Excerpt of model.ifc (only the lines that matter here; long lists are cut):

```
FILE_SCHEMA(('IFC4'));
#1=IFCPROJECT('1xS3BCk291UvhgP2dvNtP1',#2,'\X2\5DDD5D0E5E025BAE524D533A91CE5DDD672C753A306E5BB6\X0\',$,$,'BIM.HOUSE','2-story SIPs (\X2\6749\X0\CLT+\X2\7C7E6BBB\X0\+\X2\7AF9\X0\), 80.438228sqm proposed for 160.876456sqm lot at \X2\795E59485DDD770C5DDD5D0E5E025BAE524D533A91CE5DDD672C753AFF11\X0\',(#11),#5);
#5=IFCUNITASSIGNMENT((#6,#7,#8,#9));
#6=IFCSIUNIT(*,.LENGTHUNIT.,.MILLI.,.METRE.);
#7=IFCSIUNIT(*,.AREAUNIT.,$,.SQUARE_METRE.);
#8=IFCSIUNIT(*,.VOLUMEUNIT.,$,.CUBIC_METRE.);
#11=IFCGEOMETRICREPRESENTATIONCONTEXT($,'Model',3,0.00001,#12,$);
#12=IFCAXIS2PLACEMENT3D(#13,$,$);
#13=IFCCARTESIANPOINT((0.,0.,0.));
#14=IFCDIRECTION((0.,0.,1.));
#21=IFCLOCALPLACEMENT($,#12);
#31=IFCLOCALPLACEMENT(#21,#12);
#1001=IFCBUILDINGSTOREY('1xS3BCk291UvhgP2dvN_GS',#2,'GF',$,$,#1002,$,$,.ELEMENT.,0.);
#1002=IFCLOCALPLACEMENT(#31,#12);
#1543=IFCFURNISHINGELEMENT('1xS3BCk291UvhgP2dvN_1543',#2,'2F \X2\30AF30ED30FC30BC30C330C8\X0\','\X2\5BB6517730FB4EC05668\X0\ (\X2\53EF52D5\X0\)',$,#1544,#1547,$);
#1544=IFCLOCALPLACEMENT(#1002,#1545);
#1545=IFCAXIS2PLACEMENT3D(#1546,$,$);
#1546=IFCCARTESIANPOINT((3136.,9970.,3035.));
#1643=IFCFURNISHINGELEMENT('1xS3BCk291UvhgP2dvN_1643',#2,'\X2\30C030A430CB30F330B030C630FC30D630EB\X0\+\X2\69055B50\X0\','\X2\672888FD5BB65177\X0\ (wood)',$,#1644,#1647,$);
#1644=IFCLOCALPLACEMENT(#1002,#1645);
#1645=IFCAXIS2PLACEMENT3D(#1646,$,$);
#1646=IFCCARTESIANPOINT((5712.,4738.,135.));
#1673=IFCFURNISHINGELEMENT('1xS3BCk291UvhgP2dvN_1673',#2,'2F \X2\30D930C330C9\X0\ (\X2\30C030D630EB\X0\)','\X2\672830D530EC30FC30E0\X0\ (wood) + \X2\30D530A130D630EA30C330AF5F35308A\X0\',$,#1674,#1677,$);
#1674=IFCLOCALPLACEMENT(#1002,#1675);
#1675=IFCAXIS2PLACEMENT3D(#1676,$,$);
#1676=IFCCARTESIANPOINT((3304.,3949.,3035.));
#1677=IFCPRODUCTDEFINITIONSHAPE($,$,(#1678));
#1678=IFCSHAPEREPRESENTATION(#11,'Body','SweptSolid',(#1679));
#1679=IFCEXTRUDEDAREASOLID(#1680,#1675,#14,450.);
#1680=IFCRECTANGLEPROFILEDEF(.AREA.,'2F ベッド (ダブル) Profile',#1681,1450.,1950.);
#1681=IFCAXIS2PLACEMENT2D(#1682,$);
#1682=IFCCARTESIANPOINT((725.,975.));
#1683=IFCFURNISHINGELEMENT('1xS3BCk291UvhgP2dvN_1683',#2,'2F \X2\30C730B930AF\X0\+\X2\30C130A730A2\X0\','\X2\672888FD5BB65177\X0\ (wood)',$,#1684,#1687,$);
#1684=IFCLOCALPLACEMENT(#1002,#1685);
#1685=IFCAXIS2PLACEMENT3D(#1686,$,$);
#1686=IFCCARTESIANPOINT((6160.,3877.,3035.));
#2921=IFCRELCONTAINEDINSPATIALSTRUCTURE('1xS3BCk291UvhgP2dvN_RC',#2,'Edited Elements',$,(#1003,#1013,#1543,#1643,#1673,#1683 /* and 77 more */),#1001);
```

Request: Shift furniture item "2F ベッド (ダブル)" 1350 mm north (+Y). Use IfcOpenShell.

```python
import ifcopenshell
import ifcopenshell.api.geometry
import ifcopenshell.util.placement
import ifcopenshell.util.unit

model = ifcopenshell.open("model.ifc")
unit_scale = ifcopenshell.util.unit.calculate_unit_scale(model)

item = model.by_guid("1xS3BCk291UvhgP2dvN_1673")
matrix = ifcopenshell.util.placement.get_local_placement(item.ObjectPlacement)
matrix[1, 3] += 1.35 / unit_scale
ifcopenshell.api.geometry.edit_object_placement(model, product=item, matrix=matrix, is_si=False)

print(ifcopenshell.util.placement.get_local_placement(item.ObjectPlacement).round(3) + 0.0)

model.write("model_v2.ifc")
```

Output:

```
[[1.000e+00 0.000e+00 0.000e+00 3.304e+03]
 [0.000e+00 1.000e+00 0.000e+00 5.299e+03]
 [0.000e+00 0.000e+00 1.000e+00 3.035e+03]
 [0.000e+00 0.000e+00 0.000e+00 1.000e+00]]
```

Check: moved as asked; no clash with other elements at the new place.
